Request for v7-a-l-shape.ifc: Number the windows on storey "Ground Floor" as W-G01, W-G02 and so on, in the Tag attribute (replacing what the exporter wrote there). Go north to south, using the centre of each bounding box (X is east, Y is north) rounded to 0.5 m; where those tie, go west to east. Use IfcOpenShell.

First a look at what the model holds.

```python
import ifcopenshell
import ifcopenshell.util.element
import ifcopenshell.util.placement

model = ifcopenshell.open("v7-a-l-shape.ifc")
print(model.schema)
storey = next(s for s in model.by_type("IfcBuildingStorey") if s.Name == "Ground Floor")
windows = [e for e in ifcopenshell.util.element.get_decomposition(storey) if e.is_a("IfcWindow")]
for e in sorted(windows, key=lambda e: e.id()):
    origin = ifcopenshell.util.placement.get_local_placement(e.ObjectPlacement)[:3, 3]
    print(e.id(), e.Tag, e.Name, origin.round(2) + 0.0, sep=" | ")
```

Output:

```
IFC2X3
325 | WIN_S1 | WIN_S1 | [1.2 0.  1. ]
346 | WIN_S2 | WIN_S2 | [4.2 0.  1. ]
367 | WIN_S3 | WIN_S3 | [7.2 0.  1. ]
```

```python
import ifcopenshell
import ifcopenshell.geom
import ifcopenshell.util.element
import ifcopenshell.util.shape

model = ifcopenshell.open("v7-a-l-shape.ifc")
settings = ifcopenshell.geom.settings()
settings.set("use-world-coords", True)


def centre(element):
    shape = ifcopenshell.geom.create_shape(settings, element)
    return ifcopenshell.util.shape.get_bbox_centroid(shape.geometry)


storey = next(s for s in model.by_type("IfcBuildingStorey") if s.Name == "Ground Floor")
windows = [e for e in ifcopenshell.util.element.get_decomposition(storey) if e.is_a("IfcWindow")]

# Insertion points can sit at a corner or the storey origin, so sort by the geometry (in metres).
centres = {e: centre(e) for e in windows}
windows.sort(key=lambda e: (-round(centres[e][1] / 0.5), centres[e][0]))

for i, e in enumerate(windows, start=1):
    number = f"W-G{i:02d}"
    e.Tag = number
    print(e.id(), number)

model.write("v7-a-l-shape_updated.ifc")
```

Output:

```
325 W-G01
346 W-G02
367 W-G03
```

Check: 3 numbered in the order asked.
